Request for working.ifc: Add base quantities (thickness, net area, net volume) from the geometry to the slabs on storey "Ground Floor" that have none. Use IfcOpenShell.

First a look at what the model holds.

```python
import ifcopenshell
import ifcopenshell.util.element
import ifcopenshell.util.unit

model = ifcopenshell.open("working.ifc")
print(model.schema)
for unit_type in ("LENGTHUNIT", "AREAUNIT", "VOLUMEUNIT"):
    print(unit_type, ifcopenshell.util.unit.calculate_unit_scale(model, unit_type))
storey = next(s for s in model.by_type("IfcBuildingStorey") if s.Name == "Ground Floor")
slabs = [e for e in ifcopenshell.util.element.get_decomposition(storey) if e.is_a("IfcSlab")]
for e in sorted(slabs, key=lambda e: e.id()):
    print(e.id(), e.is_a(), e.Name, list(ifcopenshell.util.element.get_psets(e, qtos_only=True)), sep=" | ")
```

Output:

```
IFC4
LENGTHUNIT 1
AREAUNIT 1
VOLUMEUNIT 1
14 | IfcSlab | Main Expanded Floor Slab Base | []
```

```python
import ifcopenshell
import ifcopenshell.api.pset
import ifcopenshell.geom
import ifcopenshell.util.element
import ifcopenshell.util.shape
import ifcopenshell.util.unit

model = ifcopenshell.open("working.ifc")
unit_scale = ifcopenshell.util.unit.calculate_unit_scale(model)
area_scale = ifcopenshell.util.unit.calculate_unit_scale(model, "AREAUNIT")
volume_scale = ifcopenshell.util.unit.calculate_unit_scale(model, "VOLUMEUNIT")
settings = ifcopenshell.geom.settings()

storey = next(s for s in model.by_type("IfcBuildingStorey") if s.Name == "Ground Floor")
slabs = [e for e in ifcopenshell.util.element.get_decomposition(storey) if e.is_a("IfcSlab")]

for e in sorted(slabs, key=lambda e: e.id()):
    if ifcopenshell.util.element.get_psets(e, qtos_only=True, should_inherit=False):
        continue
    # Geometry comes back in metres, in the element's own axes.
    shape = ifcopenshell.geom.create_shape(settings, e)
    values = {
        "Width": ifcopenshell.util.shape.get_z(shape.geometry) / unit_scale,
        "NetArea": ifcopenshell.util.shape.get_footprint_area(shape.geometry) / area_scale,
        "NetVolume": ifcopenshell.util.shape.get_volume(shape.geometry) / volume_scale,
    }
    qto = ifcopenshell.api.pset.add_qto(model, product=e, name="Qto_SlabBaseQuantities")
    ifcopenshell.api.pset.edit_qto(model, qto=qto, properties=values)
    print(e.id(), {k: round(v, 3) for k, v in values.items()})

model.write("working_v2.ifc")
```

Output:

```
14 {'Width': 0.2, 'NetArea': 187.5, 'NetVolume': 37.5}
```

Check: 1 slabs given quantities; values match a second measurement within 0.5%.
